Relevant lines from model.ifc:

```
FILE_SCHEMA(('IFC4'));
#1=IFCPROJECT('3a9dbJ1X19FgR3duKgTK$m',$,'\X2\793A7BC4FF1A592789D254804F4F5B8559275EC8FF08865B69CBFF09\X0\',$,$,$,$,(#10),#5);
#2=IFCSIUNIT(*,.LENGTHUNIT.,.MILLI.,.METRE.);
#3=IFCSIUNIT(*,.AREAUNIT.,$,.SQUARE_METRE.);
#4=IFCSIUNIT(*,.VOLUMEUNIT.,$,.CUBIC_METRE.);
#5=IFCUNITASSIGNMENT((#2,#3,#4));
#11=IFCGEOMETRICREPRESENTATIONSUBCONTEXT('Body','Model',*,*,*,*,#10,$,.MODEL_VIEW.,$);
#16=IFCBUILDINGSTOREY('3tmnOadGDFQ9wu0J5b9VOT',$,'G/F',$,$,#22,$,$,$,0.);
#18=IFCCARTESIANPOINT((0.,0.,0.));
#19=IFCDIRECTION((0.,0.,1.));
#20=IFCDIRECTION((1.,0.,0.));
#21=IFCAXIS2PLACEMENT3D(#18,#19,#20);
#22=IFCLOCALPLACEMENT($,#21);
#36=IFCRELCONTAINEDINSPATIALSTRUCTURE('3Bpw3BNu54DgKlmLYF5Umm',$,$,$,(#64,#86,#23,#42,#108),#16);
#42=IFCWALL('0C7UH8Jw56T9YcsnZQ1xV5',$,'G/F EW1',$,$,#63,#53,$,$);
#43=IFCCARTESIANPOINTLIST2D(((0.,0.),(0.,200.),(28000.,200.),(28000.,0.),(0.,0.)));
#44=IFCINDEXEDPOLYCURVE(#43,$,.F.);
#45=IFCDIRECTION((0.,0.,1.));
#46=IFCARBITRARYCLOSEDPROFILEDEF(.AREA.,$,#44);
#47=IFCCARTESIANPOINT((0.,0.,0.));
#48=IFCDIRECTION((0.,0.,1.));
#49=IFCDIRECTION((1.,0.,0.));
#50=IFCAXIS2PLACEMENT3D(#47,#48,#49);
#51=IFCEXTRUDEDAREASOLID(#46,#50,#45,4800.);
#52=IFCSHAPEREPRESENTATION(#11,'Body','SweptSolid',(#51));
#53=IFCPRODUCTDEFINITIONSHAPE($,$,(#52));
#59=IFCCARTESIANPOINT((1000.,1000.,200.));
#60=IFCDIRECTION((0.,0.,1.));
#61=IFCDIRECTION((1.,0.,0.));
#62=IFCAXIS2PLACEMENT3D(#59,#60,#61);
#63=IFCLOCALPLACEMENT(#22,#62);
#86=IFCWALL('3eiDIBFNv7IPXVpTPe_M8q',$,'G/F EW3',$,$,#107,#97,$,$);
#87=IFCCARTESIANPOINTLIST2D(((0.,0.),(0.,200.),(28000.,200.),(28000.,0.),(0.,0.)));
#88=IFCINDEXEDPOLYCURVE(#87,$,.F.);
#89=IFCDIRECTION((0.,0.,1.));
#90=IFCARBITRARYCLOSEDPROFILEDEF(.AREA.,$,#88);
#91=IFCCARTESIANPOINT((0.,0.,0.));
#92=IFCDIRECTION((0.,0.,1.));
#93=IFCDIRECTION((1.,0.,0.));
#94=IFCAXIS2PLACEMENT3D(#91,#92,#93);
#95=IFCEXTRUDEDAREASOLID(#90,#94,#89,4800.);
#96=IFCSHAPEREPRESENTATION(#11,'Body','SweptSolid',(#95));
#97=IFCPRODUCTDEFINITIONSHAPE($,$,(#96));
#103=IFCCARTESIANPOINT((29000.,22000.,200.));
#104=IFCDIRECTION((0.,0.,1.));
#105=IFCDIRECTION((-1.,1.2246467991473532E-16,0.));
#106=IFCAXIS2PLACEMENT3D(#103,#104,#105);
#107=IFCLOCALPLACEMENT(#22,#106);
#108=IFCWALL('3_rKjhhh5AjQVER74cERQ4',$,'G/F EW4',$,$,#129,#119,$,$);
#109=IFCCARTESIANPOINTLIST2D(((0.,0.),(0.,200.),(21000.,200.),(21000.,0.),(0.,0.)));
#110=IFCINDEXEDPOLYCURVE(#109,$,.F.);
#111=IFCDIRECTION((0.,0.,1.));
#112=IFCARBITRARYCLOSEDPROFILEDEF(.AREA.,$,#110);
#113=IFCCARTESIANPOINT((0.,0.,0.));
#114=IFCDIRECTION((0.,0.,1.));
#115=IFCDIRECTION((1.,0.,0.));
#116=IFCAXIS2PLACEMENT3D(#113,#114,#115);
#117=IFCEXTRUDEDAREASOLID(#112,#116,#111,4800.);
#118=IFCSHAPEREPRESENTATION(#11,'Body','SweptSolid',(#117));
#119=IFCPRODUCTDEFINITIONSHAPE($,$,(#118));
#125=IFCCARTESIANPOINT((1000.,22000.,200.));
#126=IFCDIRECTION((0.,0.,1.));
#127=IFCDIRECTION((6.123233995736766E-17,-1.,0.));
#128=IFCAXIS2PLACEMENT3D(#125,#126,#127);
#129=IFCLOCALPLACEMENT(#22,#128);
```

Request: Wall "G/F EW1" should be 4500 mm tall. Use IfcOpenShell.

```python
import ifcopenshell
import ifcopenshell.geom
import ifcopenshell.util.representation
import ifcopenshell.util.shape

model = ifcopenshell.open("model.ifc")
settings = ifcopenshell.geom.settings()


def volume(element):
    """Net volume in cubic metres, openings subtracted."""
    shape = ifcopenshell.geom.create_shape(settings, element)
    return ifcopenshell.util.shape.get_volume(shape.geometry)


wall = model.by_id(42)
before = volume(wall)

body = ifcopenshell.util.representation.get_representation(wall, "Model", "Body")
solid = body.Items[0]
old_height = solid.Depth
solid.Depth = 4500.0
after = volume(wall)

print(f"height {old_height:g} -> {solid.Depth:g}, volume {before:.3f} -> {after:.3f} m3")

model.write("model_edited.ifc")
```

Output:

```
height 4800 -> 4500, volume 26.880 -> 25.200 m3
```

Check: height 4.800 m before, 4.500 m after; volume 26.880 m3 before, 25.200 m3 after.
